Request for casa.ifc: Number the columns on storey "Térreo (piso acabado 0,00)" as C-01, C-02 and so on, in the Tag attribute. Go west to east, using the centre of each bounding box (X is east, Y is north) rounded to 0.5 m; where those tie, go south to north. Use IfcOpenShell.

First a look at what the model holds.

```python
import ifcopenshell
import ifcopenshell.util.element
import ifcopenshell.util.placement

model = ifcopenshell.open("casa.ifc")
print(model.schema)
storey = next(s for s in model.by_type("IfcBuildingStorey") if s.Name == "Térreo (piso acabado 0,00)")
columns = [e for e in ifcopenshell.util.element.get_decomposition(storey) if e.is_a("IfcColumn")]
for e in sorted(columns, key=lambda e: e.id()):
    origin = ifcopenshell.util.placement.get_local_placement(e.ObjectPlacement)[:3, 3]
    print(e.id(), e.Tag, e.Name, origin.round(2) + 0.0, sep=" | ")
```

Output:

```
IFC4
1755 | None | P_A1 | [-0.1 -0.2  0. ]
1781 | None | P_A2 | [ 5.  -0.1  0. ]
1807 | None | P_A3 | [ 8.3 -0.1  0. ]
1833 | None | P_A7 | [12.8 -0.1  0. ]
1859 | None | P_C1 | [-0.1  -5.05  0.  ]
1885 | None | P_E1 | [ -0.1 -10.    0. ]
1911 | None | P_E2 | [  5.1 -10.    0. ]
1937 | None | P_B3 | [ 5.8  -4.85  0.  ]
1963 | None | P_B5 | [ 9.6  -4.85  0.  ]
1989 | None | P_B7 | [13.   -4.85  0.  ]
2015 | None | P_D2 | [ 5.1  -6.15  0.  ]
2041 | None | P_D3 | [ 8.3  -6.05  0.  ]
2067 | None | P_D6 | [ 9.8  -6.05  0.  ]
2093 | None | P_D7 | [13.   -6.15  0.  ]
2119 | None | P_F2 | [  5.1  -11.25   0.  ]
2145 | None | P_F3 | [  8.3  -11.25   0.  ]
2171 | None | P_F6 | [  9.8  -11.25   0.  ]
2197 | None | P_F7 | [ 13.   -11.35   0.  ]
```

```python
import ifcopenshell
import ifcopenshell.geom
import ifcopenshell.util.element
import ifcopenshell.util.shape

model = ifcopenshell.open("casa.ifc")
settings = ifcopenshell.geom.settings()
settings.set("use-world-coords", True)


def centre(element):
    shape = ifcopenshell.geom.create_shape(settings, element)
    return ifcopenshell.util.shape.get_bbox_centroid(shape.geometry)


storey = next(s for s in model.by_type("IfcBuildingStorey") if s.Name == "Térreo (piso acabado 0,00)")
columns = [e for e in ifcopenshell.util.element.get_decomposition(storey) if e.is_a("IfcColumn")]

# Insertion points can sit at a corner or the storey origin, so sort by the geometry (in metres).
centres = {e: centre(e) for e in columns}
columns.sort(key=lambda e: (round(centres[e][0] / 0.5), centres[e][1]))

for i, e in enumerate(columns, start=1):
    number = f"C-{i:02d}"
    e.Tag = number
    print(e.id(), number)

model.write("casa_rev.ifc")
```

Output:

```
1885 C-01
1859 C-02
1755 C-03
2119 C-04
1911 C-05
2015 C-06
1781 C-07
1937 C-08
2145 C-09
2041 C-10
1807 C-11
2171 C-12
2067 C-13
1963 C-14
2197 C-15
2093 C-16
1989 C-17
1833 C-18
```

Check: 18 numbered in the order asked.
